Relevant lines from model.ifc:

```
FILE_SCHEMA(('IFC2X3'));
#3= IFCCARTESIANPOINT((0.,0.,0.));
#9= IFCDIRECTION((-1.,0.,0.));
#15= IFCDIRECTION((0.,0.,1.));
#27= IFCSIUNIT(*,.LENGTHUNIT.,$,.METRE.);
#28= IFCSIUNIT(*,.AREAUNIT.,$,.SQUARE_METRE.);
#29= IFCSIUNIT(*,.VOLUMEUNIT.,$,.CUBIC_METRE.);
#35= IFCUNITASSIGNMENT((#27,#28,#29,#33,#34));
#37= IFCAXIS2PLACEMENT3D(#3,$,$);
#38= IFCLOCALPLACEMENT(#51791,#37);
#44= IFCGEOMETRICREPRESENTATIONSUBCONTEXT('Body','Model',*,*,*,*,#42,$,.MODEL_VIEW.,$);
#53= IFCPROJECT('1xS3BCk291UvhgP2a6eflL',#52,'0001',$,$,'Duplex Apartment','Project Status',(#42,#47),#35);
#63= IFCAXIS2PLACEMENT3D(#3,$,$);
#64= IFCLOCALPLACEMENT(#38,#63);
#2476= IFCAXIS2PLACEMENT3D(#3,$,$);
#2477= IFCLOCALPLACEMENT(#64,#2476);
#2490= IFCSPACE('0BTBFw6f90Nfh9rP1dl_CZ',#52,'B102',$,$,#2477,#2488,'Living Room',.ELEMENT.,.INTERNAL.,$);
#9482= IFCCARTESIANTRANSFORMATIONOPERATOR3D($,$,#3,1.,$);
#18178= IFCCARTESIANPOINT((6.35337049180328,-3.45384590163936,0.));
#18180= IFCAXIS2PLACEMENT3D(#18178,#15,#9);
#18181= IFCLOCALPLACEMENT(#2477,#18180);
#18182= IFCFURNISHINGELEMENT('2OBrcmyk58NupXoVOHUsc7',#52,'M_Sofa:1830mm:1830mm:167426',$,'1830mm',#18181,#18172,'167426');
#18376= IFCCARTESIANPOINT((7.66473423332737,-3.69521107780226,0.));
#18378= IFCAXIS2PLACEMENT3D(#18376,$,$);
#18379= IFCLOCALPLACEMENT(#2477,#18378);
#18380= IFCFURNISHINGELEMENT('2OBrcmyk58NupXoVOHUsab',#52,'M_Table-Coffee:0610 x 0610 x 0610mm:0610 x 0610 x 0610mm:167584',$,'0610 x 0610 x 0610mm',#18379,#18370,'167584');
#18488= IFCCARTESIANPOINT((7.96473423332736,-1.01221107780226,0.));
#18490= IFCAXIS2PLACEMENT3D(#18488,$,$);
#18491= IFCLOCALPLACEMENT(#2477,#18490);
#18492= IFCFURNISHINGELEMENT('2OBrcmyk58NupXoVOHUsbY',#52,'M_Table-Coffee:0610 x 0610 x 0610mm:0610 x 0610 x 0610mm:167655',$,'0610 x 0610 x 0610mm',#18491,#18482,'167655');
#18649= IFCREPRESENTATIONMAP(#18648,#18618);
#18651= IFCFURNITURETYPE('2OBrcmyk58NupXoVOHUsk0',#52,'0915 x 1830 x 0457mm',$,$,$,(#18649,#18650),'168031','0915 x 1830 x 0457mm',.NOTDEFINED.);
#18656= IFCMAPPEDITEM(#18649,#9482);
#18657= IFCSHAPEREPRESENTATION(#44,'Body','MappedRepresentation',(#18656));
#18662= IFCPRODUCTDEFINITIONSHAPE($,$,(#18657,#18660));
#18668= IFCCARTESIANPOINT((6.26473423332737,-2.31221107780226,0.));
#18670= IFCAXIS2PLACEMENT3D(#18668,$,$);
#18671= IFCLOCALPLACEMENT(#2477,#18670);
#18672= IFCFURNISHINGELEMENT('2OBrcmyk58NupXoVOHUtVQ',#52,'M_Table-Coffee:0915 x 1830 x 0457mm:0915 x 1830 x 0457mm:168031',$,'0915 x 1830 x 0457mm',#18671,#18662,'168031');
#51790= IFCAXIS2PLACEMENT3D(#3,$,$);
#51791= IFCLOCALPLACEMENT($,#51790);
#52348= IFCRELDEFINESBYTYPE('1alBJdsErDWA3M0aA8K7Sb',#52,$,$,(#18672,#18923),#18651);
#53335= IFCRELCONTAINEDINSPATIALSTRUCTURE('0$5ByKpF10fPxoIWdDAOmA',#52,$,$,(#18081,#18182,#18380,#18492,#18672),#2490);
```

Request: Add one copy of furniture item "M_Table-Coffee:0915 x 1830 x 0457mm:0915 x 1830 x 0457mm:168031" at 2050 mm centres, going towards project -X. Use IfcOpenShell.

```python
import numpy as np
import ifcopenshell
import ifcopenshell.api.geometry
import ifcopenshell.api.root
import ifcopenshell.util.element
import ifcopenshell.util.placement

model = ifcopenshell.open("model.ifc")


def reuse_history(source, copy):
    """copy_class also copies each property set's owner history, people and application; keep the originals."""
    for rel in copy.IsDefinedBy:
        if rel.is_a("IfcRelDefinesByProperties") and (history := rel.RelatingPropertyDefinition.OwnerHistory):
            rel.RelatingPropertyDefinition.OwnerHistory = source.OwnerHistory
            ifcopenshell.util.element.remove_deep2(model, history)


source = model.by_guid("2OBrcmyk58NupXoVOHUtVQ")
base = ifcopenshell.util.placement.get_local_placement(source.ObjectPlacement)
step = np.array([-1.0, 0.0, 0.0]) * 2.05

for i in range(1, 2):
    copy = ifcopenshell.api.root.copy_class(model, product=source)
    copy.Representation = ifcopenshell.util.element.copy_deep(
        model, source.Representation, exclude=["IfcGeometricRepresentationContext", "IfcRepresentationMap"]
    )
    copy.Name = "M_Table-Coffee:0915 x 1830 x 0457mm:0915 x 1830 x 0457mm"
    copy.Tag = None
    reuse_history(source, copy)
    matrix = base.copy()
    matrix[:3, 3] += i * step
    print("added at", matrix[:3, 3].round(3) + 0.0)
    ifcopenshell.api.geometry.edit_object_placement(model, product=copy, matrix=matrix, is_si=False)

model.write("model-out.ifc")
```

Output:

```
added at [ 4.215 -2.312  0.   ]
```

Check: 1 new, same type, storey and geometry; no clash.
